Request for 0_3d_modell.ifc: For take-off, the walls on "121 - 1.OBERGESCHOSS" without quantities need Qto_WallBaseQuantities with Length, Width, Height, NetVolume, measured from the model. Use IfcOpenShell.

First a look at what the model holds.

```python
import ifcopenshell
import ifcopenshell.util.element
import ifcopenshell.util.unit

model = ifcopenshell.open("0_3d_modell.ifc")
print(model.schema)
for unit_type in ("LENGTHUNIT", "AREAUNIT", "VOLUMEUNIT"):
    print(unit_type, ifcopenshell.util.unit.calculate_unit_scale(model, unit_type))
storey = next(s for s in model.by_type("IfcBuildingStorey") if s.Name == "121 - 1.OBERGESCHOSS")
walls = [e for e in ifcopenshell.util.element.get_decomposition(storey) if e.is_a("IfcWall")]
for e in sorted(walls, key=lambda e: e.id()):
    print(e.id(), e.is_a(), e.Name, list(ifcopenshell.util.element.get_psets(e, qtos_only=True)), sep=" | ")
```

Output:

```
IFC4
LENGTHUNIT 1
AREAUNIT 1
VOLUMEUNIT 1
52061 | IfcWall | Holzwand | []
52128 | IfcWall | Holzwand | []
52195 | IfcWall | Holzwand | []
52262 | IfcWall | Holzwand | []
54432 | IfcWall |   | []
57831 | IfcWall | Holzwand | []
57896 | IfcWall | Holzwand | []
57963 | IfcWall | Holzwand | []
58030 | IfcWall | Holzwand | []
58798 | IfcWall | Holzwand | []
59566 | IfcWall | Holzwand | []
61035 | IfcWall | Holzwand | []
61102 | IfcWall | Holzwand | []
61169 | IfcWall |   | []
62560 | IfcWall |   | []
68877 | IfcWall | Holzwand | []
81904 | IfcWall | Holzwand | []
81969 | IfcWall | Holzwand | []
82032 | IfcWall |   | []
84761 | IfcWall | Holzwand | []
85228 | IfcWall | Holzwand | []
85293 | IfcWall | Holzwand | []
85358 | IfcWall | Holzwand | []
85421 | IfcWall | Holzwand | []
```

```python
import ifcopenshell
import ifcopenshell.api.pset
import ifcopenshell.geom
import ifcopenshell.util.element
import ifcopenshell.util.shape
import ifcopenshell.util.unit

model = ifcopenshell.open("0_3d_modell.ifc")
unit_scale = ifcopenshell.util.unit.calculate_unit_scale(model)
volume_scale = ifcopenshell.util.unit.calculate_unit_scale(model, "VOLUMEUNIT")
settings = ifcopenshell.geom.settings()

storey = next(s for s in model.by_type("IfcBuildingStorey") if s.Name == "121 - 1.OBERGESCHOSS")
walls = [e for e in ifcopenshell.util.element.get_decomposition(storey) if e.is_a("IfcWall")]

for e in sorted(walls, key=lambda e: e.id()):
    if ifcopenshell.util.element.get_psets(e, qtos_only=True, should_inherit=False):
        continue
    # Geometry comes back in metres, in the element's own axes.
    shape = ifcopenshell.geom.create_shape(settings, e)
    values = {
        "Length": ifcopenshell.util.shape.get_x(shape.geometry) / unit_scale,
        "Width": ifcopenshell.util.shape.get_y(shape.geometry) / unit_scale,
        "Height": ifcopenshell.util.shape.get_z(shape.geometry) / unit_scale,
        "NetVolume": ifcopenshell.util.shape.get_volume(shape.geometry) / volume_scale,
    }
    qto = ifcopenshell.api.pset.add_qto(model, product=e, name="Qto_WallBaseQuantities")
    ifcopenshell.api.pset.edit_qto(model, qto=qto, properties=values)
    print(e.id(), {k: round(v, 3) for k, v in values.items()})

model.write("0_3d_modell-out.ifc")
```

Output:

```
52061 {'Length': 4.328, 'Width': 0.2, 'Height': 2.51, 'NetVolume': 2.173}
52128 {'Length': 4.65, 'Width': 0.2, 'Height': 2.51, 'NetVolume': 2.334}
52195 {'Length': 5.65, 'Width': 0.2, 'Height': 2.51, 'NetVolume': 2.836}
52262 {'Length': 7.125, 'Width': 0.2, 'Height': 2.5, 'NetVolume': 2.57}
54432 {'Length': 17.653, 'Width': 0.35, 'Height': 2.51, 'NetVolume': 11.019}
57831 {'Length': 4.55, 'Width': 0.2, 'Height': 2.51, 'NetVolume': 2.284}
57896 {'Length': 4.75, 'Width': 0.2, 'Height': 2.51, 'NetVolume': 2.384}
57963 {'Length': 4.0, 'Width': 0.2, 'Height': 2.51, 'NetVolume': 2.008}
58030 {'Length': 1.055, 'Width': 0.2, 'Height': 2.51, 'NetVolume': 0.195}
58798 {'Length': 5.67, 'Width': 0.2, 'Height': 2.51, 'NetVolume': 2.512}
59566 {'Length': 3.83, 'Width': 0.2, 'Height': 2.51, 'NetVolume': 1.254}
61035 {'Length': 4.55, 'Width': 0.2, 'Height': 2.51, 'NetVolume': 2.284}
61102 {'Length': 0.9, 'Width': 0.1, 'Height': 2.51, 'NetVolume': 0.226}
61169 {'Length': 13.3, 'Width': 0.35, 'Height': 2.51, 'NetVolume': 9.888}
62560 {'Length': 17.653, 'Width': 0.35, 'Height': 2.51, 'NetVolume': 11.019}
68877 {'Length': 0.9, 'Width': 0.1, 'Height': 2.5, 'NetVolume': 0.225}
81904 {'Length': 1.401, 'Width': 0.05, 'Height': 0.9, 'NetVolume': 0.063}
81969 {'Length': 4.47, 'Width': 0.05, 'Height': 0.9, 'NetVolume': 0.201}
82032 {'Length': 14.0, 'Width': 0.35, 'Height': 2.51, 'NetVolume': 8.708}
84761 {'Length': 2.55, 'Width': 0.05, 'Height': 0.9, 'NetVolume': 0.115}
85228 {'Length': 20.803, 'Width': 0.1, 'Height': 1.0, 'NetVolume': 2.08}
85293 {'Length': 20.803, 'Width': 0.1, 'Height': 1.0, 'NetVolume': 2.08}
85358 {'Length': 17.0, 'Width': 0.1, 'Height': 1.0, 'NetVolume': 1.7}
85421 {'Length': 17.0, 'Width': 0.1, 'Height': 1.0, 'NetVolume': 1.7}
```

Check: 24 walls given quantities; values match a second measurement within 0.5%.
